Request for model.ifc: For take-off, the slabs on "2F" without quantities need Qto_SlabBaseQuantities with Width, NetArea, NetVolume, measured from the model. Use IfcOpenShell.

First a look at what the model holds.

```python
import ifcopenshell
import ifcopenshell.util.element
import ifcopenshell.util.unit

model = ifcopenshell.open("model.ifc")
print(model.schema)
for unit_type in ("LENGTHUNIT", "AREAUNIT", "VOLUMEUNIT"):
    print(unit_type, ifcopenshell.util.unit.calculate_unit_scale(model, unit_type))
storey = next(s for s in model.by_type("IfcBuildingStorey") if s.Name == "2F")
slabs = [e for e in ifcopenshell.util.element.get_decomposition(storey) if e.is_a("IfcSlab")]
for e in sorted(slabs, key=lambda e: e.id()):
    print(e.id(), e.is_a(), e.Name, list(ifcopenshell.util.element.get_psets(e, qtos_only=True)), sep=" | ")
```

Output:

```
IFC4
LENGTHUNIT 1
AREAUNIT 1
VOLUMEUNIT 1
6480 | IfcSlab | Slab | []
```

```python
import ifcopenshell
import ifcopenshell.api.pset
import ifcopenshell.geom
import ifcopenshell.util.element
import ifcopenshell.util.shape
import ifcopenshell.util.unit

model = ifcopenshell.open("model.ifc")
unit_scale = ifcopenshell.util.unit.calculate_unit_scale(model)
area_scale = ifcopenshell.util.unit.calculate_unit_scale(model, "AREAUNIT")
volume_scale = ifcopenshell.util.unit.calculate_unit_scale(model, "VOLUMEUNIT")
settings = ifcopenshell.geom.settings()

storey = next(s for s in model.by_type("IfcBuildingStorey") if s.Name == "2F")
slabs = [e for e in ifcopenshell.util.element.get_decomposition(storey) if e.is_a("IfcSlab")]

for e in sorted(slabs, key=lambda e: e.id()):
    if ifcopenshell.util.element.get_psets(e, qtos_only=True, should_inherit=False):
        continue
    # Geometry comes back in metres, in the element's own axes.
    shape = ifcopenshell.geom.create_shape(settings, e)
    values = {
        "Width": ifcopenshell.util.shape.get_z(shape.geometry) / unit_scale,
        "NetArea": ifcopenshell.util.shape.get_footprint_area(shape.geometry) / area_scale,
        "NetVolume": ifcopenshell.util.shape.get_volume(shape.geometry) / volume_scale,
    }
    qto = ifcopenshell.api.pset.add_qto(model, product=e, name="Qto_SlabBaseQuantities")
    ifcopenshell.api.pset.edit_qto(model, qto=qto, properties=values)
    print(e.id(), {k: round(v, 3) for k, v in values.items()})

model.write("model_updated.ifc")
```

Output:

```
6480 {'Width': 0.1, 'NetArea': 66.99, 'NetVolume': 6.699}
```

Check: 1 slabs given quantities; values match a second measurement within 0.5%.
